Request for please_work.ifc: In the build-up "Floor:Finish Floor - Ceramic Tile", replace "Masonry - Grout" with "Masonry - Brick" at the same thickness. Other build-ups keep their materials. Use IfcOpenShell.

First a look at what the model holds.

```python
import ifcopenshell
import ifcopenshell.util.element

model = ifcopenshell.open("please_work.ifc")
print(model.schema)
for layer_set in model.by_type("IfcMaterialLayerSet"):
    if layer_set.LayerSetName == "Floor:Finish Floor - Ceramic Tile":
        for layer in layer_set.MaterialLayers:
            print(layer.id(), layer.Material and layer.Material.Name, layer.LayerThickness, sep=" | ")
        print(len(ifcopenshell.util.element.get_elements_by_material(model, layer_set)), "elements and types use it")
print(sorted(m.Name for m in model.by_type("IfcMaterial") if m.Name)[:60])
```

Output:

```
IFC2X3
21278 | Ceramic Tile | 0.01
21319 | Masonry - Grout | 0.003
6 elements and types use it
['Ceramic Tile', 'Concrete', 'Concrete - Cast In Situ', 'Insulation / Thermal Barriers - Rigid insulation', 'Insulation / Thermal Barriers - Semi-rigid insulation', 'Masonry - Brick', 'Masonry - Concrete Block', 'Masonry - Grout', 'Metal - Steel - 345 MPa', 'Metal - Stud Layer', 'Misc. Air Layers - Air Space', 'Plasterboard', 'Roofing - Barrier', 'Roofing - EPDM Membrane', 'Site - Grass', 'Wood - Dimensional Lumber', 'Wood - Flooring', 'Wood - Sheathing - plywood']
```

```python
import ifcopenshell
import ifcopenshell.api.material

model = ifcopenshell.open("please_work.ifc")

layer_set = next(s for s in model.by_type("IfcMaterialLayerSet") if s.LayerSetName == "Floor:Finish Floor - Ceramic Tile")
layer = next(l for l in layer_set.MaterialLayers if l.Material and l.Material.Name == "Masonry - Grout")
material = next(m for m in model.by_type("IfcMaterial") if m.Name == "Masonry - Brick")

# Point this one layer at the other material; renaming the old one would change it everywhere.
ifcopenshell.api.material.edit_layer(model, layer=layer, attributes={}, material=material)

print([l.Material.Name if l.Material else None for l in layer_set.MaterialLayers])

model.write("please_work_v2.ifc")
```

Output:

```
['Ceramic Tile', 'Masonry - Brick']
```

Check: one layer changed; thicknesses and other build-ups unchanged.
